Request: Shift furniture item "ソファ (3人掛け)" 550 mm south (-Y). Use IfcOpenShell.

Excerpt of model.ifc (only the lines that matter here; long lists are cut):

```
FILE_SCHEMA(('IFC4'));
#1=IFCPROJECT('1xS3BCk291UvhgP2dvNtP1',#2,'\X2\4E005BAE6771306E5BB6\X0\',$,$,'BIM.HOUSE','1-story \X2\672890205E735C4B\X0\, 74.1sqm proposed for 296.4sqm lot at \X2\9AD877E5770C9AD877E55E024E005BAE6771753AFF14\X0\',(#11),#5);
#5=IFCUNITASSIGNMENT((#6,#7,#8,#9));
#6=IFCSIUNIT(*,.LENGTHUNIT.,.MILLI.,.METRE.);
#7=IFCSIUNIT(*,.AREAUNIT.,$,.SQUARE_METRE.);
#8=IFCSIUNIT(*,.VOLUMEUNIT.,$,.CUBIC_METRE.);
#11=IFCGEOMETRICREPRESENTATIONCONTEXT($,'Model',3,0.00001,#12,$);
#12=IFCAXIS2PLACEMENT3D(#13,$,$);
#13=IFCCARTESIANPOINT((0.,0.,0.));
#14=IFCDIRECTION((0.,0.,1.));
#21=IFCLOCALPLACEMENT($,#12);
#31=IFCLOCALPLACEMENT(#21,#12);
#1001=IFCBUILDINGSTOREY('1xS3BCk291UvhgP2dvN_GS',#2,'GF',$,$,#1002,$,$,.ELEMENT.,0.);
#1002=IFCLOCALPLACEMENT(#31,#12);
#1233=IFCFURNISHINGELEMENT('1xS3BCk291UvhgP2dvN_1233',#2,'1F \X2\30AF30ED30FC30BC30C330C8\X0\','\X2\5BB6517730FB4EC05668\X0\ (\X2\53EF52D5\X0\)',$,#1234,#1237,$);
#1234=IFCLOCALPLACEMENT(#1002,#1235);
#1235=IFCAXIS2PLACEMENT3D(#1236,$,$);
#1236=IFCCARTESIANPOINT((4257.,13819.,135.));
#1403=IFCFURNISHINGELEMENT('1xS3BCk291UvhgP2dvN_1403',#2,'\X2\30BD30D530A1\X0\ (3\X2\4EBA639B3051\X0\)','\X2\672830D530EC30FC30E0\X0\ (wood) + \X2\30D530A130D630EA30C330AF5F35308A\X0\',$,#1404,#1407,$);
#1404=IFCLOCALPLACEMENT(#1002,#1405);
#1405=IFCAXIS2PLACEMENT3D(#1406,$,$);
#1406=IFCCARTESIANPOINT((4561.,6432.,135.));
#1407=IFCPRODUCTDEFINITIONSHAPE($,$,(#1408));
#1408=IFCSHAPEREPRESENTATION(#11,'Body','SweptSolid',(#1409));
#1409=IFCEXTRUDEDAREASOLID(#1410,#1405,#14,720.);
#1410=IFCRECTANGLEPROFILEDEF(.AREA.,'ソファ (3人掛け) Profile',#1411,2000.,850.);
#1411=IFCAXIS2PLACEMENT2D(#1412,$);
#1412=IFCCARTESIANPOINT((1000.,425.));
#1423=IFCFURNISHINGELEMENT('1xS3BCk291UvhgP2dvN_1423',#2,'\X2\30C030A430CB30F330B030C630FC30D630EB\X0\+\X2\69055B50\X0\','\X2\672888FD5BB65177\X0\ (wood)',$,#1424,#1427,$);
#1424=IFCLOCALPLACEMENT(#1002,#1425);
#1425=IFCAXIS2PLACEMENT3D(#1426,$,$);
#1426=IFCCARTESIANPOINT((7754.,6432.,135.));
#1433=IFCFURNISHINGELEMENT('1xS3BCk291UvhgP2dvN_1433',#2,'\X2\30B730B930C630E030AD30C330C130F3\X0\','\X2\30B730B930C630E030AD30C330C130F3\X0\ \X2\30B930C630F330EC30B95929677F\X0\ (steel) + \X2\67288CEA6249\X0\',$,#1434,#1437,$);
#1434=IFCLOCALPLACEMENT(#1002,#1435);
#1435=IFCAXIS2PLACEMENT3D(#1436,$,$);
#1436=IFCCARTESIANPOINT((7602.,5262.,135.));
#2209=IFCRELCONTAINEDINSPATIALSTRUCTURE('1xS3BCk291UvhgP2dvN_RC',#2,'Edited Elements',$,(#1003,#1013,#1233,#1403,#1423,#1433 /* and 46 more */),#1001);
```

```python
import ifcopenshell
import ifcopenshell.api.geometry
import ifcopenshell.util.placement
import ifcopenshell.util.unit

model = ifcopenshell.open("model.ifc")
unit_scale = ifcopenshell.util.unit.calculate_unit_scale(model)

item = model.by_guid("1xS3BCk291UvhgP2dvN_1403")
matrix = ifcopenshell.util.placement.get_local_placement(item.ObjectPlacement)
matrix[1, 3] -= 0.55 / unit_scale
ifcopenshell.api.geometry.edit_object_placement(model, product=item, matrix=matrix, is_si=False)

print(ifcopenshell.util.placement.get_local_placement(item.ObjectPlacement).round(3) + 0.0)

model.write("model_v2.ifc")
```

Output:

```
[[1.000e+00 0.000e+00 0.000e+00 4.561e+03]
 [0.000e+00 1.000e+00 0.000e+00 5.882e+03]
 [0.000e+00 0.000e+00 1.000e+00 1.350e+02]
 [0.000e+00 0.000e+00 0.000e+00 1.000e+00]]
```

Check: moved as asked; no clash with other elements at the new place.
